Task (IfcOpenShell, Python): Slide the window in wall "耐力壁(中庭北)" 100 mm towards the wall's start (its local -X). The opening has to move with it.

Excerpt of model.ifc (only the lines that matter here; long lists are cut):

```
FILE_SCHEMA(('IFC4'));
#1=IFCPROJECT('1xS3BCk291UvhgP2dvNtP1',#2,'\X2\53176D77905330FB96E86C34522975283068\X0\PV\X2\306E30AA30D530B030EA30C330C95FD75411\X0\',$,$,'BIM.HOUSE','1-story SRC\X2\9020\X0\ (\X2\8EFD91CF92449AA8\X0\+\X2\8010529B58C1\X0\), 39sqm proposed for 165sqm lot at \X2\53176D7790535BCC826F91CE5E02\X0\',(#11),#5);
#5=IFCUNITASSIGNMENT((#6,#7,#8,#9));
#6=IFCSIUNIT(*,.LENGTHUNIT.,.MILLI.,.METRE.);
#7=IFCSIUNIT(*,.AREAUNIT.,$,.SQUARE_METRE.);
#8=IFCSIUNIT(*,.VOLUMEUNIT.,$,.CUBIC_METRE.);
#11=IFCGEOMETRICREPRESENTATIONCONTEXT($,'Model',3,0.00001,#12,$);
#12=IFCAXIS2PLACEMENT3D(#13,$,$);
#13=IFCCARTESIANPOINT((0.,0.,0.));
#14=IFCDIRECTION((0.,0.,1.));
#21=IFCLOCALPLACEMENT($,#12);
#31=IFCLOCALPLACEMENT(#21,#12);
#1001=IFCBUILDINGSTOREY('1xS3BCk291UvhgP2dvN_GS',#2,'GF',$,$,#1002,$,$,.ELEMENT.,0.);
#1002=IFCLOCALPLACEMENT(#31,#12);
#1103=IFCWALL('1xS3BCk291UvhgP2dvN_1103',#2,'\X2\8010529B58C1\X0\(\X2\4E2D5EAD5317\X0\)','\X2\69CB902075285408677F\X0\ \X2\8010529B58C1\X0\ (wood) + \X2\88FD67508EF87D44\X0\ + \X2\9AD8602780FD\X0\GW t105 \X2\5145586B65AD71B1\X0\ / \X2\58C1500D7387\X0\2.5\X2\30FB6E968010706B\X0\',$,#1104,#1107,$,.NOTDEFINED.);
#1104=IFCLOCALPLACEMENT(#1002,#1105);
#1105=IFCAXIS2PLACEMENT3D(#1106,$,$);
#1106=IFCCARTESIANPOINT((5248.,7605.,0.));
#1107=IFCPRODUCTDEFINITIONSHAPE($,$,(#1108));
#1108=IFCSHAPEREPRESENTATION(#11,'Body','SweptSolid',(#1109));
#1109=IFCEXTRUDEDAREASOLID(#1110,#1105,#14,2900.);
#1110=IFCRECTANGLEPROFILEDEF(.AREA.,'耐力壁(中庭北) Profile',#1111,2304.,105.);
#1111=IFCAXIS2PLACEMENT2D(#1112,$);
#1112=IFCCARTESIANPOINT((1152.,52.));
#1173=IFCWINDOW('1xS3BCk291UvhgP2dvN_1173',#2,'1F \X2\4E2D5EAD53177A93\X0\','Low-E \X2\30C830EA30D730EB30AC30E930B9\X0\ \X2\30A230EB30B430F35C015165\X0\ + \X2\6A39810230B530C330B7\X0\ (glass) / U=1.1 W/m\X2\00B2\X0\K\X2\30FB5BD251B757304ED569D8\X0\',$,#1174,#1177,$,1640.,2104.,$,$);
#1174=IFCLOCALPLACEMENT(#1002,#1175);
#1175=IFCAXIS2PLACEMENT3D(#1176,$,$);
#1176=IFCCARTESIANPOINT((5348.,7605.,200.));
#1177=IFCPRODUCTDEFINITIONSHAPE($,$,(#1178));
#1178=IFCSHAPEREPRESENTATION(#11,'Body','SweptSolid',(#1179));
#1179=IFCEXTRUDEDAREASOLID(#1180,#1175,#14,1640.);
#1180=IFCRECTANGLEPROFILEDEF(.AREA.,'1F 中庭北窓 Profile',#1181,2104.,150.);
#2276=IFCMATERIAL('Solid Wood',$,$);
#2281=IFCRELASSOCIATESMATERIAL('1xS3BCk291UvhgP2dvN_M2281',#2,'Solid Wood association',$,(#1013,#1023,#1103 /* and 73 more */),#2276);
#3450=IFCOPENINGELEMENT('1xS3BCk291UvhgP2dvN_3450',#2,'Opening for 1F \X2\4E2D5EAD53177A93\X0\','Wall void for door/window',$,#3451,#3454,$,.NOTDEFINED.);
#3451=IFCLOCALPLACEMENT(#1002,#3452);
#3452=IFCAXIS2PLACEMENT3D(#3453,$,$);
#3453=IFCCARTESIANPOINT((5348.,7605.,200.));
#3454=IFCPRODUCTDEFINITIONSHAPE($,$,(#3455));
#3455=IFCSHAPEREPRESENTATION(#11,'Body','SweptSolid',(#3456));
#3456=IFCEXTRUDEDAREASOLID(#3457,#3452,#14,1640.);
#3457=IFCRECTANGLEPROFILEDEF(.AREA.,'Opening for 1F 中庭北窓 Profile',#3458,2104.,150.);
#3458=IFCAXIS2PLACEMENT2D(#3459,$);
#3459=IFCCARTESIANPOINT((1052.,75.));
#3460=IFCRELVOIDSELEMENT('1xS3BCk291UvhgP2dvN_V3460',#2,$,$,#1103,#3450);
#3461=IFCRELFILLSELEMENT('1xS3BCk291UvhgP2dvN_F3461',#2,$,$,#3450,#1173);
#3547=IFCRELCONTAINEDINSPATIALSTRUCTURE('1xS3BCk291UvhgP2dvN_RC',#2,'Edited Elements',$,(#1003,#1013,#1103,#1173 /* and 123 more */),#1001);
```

```python
import ifcopenshell
import ifcopenshell.api.geometry
import ifcopenshell.util.placement
import ifcopenshell.util.unit

model = ifcopenshell.open("model.ifc")
unit_scale = ifcopenshell.util.unit.calculate_unit_scale(model)

window = model.by_guid("1xS3BCk291UvhgP2dvN_1173")
opening = window.FillsVoids[0].RelatingOpeningElement
wall = opening.VoidsElements[0].RelatingBuildingElement

wall_matrix = ifcopenshell.util.placement.get_local_placement(wall.ObjectPlacement)
shift = wall_matrix[:3, 0] * -0.1 / unit_scale
before = ifcopenshell.util.placement.get_local_placement(window.ObjectPlacement)[:3, 3].copy()

# The window is not placed relative to its opening, so move both.
for product in (opening, window):
    matrix = ifcopenshell.util.placement.get_local_placement(product.ObjectPlacement)
    matrix[:3, 3] += shift
    ifcopenshell.api.geometry.edit_object_placement(model, product=product, matrix=matrix, is_si=False)

after = ifcopenshell.util.placement.get_local_placement(window.ObjectPlacement)[:3, 3]
print("window moved by", (after - before).round(3) + 0.0)

model.write("model-out.ifc")
```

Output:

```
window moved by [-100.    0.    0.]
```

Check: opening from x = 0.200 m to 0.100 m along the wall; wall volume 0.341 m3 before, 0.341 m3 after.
